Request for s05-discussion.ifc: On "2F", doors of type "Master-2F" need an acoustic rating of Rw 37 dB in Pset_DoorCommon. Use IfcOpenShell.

First a look at what the model holds.

```python
import ifcopenshell
import ifcopenshell.util.element

model = ifcopenshell.open("s05-discussion.ifc")
print(model.schema)
storey = next(s for s in model.by_type("IfcBuildingStorey") if s.Name == "2F")
doors = [e for e in ifcopenshell.util.element.get_decomposition(storey) if e.is_a("IfcDoor")]
seen = {}
for e in doors:
    element_type = ifcopenshell.util.element.get_type(e)
    key = (element_type.Name if element_type != e and element_type else None, ifcopenshell.util.element.get_pset(e, "Pset_DoorCommon", "AcousticRating"))
    seen[key] = seen.get(key, 0) + 1
for (name, value), count in sorted(seen.items(), key=str):
    print(count, "x", name, "|", value)
```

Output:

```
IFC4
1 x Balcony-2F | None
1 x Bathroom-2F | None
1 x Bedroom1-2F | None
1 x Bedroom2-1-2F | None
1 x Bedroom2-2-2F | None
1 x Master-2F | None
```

```python
import ifcopenshell
import ifcopenshell.api.pset
import ifcopenshell.util.element

model = ifcopenshell.open("s05-discussion.ifc")

storey = next(s for s in model.by_type("IfcBuildingStorey") if s.Name == "2F")
doors = [e for e in ifcopenshell.util.element.get_decomposition(storey) if e.is_a("IfcDoor")]

count = 0
for e in doors:
    element_type = ifcopenshell.util.element.get_type(e)
    if element_type in (None, e) or element_type.Name != "Master-2F":
        continue
    # add_pset returns the element's existing set when there is one.
    pset = ifcopenshell.api.pset.add_pset(model, product=e, name="Pset_DoorCommon")
    ifcopenshell.api.pset.edit_pset(model, pset=pset, properties={"AcousticRating": "Rw 37 dB"})
    count += 1

print(count, "doors updated")

model.write("s05-discussion_v2.ifc")
```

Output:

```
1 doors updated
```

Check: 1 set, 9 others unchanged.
